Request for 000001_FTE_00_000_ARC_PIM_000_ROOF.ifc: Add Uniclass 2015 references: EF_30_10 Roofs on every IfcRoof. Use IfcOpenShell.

First a look at what the model holds.

```python
import ifcopenshell

model = ifcopenshell.open("000001_FTE_00_000_ARC_PIM_000_ROOF.ifc")
print(model.schema)
print("classifications:", [c.Name for c in model.by_type("IfcClassification")])
for ifc_class in ("IfcDoor", "IfcRoof", "IfcStair", "IfcWall", "IfcWindow"):
    print(ifc_class, len(model.by_type(ifc_class)))
```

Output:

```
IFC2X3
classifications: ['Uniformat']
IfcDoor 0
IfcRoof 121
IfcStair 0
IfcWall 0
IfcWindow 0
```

```python
import ifcopenshell
import ifcopenshell.api.classification

model = ifcopenshell.open("000001_FTE_00_000_ARC_PIM_000_ROOF.ifc")

# IFC2X3 requires Source and Edition and has no link from the project to the system.
system = model.create_entity("IfcClassification", Source="NBS", Edition="2015", Name="Uniclass 2015")

codes = {
    "IfcRoof": ("EF_30_10", "Roofs"),
}
for ifc_class, (code, name) in codes.items():
    products = model.by_type(ifc_class)
    ifcopenshell.api.classification.add_reference(
        model, products=products, classification=system, identification=code, name=name
    )
    print(code, len(products))

model.write("000001_FTE_00_000_ARC_PIM_000_ROOF-out.ifc")
```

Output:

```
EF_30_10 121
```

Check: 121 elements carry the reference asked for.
